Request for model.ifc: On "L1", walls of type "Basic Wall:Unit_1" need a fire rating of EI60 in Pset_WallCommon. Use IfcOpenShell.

First a look at what the model holds.

```python
import ifcopenshell
import ifcopenshell.util.element

model = ifcopenshell.open("model.ifc")
print(model.schema)
storey = next(s for s in model.by_type("IfcBuildingStorey") if s.Name == "L1")
walls = [e for e in ifcopenshell.util.element.get_decomposition(storey) if e.is_a("IfcWall")]
seen = {}
for e in walls:
    element_type = ifcopenshell.util.element.get_type(e)
    key = (element_type.Name if element_type != e and element_type else None, ifcopenshell.util.element.get_pset(e, "Pset_WallCommon", "FireRating"))
    seen[key] = seen.get(key, 0) + 1
for (name, value), count in sorted(seen.items(), key=str):
    print(count, "x", name, "|", value)
```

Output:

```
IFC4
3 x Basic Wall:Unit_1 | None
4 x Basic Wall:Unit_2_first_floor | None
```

```python
import ifcopenshell
import ifcopenshell.api.pset
import ifcopenshell.util.element

model = ifcopenshell.open("model.ifc")

storey = next(s for s in model.by_type("IfcBuildingStorey") if s.Name == "L1")
walls = [e for e in ifcopenshell.util.element.get_decomposition(storey) if e.is_a("IfcWall")]

count = 0
for e in walls:
    element_type = ifcopenshell.util.element.get_type(e)
    if element_type in (None, e) or element_type.Name != "Basic Wall:Unit_1":
        continue
    # add_pset returns the element's existing set when there is one.
    pset = ifcopenshell.api.pset.add_pset(model, product=e, name="Pset_WallCommon")
    ifcopenshell.api.pset.edit_pset(model, pset=pset, properties={"FireRating": "EI60"})
    count += 1

print(count, "walls updated")

model.write("model_updated.ifc")
```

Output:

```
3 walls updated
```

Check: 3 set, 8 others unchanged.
